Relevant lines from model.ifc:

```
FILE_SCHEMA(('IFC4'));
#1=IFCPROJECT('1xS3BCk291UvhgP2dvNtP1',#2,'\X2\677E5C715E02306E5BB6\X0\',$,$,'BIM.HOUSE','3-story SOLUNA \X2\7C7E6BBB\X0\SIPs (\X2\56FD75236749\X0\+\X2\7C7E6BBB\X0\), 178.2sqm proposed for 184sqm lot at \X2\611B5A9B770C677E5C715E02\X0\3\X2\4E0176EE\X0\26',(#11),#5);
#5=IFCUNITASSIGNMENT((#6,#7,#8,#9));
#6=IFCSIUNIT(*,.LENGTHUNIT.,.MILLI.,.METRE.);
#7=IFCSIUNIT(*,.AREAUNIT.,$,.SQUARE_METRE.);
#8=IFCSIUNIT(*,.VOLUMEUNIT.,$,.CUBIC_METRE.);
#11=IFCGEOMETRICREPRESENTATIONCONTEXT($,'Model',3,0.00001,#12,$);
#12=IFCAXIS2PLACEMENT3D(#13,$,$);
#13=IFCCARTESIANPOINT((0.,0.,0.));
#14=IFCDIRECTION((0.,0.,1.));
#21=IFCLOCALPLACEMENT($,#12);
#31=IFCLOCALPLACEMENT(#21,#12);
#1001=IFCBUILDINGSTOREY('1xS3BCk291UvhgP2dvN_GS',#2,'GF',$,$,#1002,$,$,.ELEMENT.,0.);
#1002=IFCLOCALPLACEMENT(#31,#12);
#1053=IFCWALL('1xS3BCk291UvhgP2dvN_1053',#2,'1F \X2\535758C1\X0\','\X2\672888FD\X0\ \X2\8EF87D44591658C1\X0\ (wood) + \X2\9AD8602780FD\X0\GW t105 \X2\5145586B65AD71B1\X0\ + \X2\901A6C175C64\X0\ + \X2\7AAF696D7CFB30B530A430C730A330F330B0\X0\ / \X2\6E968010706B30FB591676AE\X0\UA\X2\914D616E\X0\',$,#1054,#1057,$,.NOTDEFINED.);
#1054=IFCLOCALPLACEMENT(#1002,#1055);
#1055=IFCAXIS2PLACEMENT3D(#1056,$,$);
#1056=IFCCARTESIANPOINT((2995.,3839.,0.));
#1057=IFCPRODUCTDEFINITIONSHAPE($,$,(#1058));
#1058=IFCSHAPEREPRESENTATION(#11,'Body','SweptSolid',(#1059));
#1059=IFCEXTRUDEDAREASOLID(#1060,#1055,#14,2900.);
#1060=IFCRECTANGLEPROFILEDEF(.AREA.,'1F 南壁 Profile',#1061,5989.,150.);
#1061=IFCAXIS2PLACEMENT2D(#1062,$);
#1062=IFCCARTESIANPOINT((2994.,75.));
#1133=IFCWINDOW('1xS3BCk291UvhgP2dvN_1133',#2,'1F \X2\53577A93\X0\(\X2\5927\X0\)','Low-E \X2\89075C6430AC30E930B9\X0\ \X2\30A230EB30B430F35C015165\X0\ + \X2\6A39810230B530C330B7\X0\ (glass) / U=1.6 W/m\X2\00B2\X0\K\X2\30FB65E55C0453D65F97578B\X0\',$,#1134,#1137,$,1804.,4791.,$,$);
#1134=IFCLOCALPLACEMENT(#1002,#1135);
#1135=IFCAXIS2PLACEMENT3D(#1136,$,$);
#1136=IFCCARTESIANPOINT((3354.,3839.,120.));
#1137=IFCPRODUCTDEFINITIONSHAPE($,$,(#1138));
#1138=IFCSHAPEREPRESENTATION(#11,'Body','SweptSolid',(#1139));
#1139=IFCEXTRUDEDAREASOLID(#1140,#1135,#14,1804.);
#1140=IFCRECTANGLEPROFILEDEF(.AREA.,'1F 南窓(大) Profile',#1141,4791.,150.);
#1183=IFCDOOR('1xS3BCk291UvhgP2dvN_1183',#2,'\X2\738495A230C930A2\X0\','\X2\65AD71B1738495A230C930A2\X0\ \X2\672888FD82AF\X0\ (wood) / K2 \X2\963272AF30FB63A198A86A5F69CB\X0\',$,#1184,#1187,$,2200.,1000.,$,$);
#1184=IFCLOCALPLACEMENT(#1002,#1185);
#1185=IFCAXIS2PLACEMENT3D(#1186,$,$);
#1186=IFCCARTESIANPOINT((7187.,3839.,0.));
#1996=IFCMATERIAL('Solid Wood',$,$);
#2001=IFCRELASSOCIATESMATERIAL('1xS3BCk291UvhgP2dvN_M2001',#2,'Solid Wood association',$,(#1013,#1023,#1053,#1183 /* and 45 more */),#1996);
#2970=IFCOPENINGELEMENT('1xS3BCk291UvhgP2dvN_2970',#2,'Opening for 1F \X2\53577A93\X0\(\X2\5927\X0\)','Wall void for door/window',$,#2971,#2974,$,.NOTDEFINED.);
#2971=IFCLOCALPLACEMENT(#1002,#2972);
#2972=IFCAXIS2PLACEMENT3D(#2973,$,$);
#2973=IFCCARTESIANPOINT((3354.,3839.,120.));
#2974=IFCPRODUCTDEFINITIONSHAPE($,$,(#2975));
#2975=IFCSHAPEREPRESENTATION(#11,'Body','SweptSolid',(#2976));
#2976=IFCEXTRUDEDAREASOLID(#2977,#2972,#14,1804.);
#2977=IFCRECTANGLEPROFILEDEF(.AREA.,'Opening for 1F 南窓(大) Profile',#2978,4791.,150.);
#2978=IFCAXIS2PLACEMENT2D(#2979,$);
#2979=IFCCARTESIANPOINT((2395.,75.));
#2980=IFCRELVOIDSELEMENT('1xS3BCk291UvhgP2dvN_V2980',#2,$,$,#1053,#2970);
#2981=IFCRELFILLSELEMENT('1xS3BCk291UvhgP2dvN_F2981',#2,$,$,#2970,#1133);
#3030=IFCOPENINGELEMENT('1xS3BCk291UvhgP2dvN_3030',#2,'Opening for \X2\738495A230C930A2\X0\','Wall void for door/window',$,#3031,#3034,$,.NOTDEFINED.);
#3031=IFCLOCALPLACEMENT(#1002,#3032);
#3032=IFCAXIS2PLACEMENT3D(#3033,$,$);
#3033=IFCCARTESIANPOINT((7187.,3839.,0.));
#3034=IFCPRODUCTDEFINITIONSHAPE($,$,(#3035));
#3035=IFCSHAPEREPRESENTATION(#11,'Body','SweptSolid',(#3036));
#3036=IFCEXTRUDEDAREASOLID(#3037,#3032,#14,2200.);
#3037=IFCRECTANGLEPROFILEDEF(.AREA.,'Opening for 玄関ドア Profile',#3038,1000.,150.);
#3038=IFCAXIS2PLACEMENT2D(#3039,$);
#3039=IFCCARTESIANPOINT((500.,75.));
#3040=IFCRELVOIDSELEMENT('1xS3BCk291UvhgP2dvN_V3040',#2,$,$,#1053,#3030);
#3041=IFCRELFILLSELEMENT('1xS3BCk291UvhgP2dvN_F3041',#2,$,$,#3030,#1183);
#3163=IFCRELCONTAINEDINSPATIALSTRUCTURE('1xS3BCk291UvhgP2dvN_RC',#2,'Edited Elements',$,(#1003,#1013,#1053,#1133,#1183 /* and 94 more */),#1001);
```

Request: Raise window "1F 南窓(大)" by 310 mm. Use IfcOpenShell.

```python
import numpy as np
import ifcopenshell
import ifcopenshell.api.geometry
import ifcopenshell.util.placement
import ifcopenshell.util.unit

model = ifcopenshell.open("model.ifc")
unit_scale = ifcopenshell.util.unit.calculate_unit_scale(model)

window = model.by_guid("1xS3BCk291UvhgP2dvN_1133")
opening = window.FillsVoids[0].RelatingOpeningElement
dz = 0.31 / unit_scale

shift = np.array([0.0, 0.0, dz])
# The window is not placed relative to its opening, so move both.
for product in (opening, window):
    matrix = ifcopenshell.util.placement.get_local_placement(product.ObjectPlacement)
    matrix[:3, 3] += shift
    ifcopenshell.api.geometry.edit_object_placement(model, product=product, matrix=matrix, is_si=False)

print(f"moved by {dz * unit_scale:+.3f} m")

model.write("model_updated.ifc")
```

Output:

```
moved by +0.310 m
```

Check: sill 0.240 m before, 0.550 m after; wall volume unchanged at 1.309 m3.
